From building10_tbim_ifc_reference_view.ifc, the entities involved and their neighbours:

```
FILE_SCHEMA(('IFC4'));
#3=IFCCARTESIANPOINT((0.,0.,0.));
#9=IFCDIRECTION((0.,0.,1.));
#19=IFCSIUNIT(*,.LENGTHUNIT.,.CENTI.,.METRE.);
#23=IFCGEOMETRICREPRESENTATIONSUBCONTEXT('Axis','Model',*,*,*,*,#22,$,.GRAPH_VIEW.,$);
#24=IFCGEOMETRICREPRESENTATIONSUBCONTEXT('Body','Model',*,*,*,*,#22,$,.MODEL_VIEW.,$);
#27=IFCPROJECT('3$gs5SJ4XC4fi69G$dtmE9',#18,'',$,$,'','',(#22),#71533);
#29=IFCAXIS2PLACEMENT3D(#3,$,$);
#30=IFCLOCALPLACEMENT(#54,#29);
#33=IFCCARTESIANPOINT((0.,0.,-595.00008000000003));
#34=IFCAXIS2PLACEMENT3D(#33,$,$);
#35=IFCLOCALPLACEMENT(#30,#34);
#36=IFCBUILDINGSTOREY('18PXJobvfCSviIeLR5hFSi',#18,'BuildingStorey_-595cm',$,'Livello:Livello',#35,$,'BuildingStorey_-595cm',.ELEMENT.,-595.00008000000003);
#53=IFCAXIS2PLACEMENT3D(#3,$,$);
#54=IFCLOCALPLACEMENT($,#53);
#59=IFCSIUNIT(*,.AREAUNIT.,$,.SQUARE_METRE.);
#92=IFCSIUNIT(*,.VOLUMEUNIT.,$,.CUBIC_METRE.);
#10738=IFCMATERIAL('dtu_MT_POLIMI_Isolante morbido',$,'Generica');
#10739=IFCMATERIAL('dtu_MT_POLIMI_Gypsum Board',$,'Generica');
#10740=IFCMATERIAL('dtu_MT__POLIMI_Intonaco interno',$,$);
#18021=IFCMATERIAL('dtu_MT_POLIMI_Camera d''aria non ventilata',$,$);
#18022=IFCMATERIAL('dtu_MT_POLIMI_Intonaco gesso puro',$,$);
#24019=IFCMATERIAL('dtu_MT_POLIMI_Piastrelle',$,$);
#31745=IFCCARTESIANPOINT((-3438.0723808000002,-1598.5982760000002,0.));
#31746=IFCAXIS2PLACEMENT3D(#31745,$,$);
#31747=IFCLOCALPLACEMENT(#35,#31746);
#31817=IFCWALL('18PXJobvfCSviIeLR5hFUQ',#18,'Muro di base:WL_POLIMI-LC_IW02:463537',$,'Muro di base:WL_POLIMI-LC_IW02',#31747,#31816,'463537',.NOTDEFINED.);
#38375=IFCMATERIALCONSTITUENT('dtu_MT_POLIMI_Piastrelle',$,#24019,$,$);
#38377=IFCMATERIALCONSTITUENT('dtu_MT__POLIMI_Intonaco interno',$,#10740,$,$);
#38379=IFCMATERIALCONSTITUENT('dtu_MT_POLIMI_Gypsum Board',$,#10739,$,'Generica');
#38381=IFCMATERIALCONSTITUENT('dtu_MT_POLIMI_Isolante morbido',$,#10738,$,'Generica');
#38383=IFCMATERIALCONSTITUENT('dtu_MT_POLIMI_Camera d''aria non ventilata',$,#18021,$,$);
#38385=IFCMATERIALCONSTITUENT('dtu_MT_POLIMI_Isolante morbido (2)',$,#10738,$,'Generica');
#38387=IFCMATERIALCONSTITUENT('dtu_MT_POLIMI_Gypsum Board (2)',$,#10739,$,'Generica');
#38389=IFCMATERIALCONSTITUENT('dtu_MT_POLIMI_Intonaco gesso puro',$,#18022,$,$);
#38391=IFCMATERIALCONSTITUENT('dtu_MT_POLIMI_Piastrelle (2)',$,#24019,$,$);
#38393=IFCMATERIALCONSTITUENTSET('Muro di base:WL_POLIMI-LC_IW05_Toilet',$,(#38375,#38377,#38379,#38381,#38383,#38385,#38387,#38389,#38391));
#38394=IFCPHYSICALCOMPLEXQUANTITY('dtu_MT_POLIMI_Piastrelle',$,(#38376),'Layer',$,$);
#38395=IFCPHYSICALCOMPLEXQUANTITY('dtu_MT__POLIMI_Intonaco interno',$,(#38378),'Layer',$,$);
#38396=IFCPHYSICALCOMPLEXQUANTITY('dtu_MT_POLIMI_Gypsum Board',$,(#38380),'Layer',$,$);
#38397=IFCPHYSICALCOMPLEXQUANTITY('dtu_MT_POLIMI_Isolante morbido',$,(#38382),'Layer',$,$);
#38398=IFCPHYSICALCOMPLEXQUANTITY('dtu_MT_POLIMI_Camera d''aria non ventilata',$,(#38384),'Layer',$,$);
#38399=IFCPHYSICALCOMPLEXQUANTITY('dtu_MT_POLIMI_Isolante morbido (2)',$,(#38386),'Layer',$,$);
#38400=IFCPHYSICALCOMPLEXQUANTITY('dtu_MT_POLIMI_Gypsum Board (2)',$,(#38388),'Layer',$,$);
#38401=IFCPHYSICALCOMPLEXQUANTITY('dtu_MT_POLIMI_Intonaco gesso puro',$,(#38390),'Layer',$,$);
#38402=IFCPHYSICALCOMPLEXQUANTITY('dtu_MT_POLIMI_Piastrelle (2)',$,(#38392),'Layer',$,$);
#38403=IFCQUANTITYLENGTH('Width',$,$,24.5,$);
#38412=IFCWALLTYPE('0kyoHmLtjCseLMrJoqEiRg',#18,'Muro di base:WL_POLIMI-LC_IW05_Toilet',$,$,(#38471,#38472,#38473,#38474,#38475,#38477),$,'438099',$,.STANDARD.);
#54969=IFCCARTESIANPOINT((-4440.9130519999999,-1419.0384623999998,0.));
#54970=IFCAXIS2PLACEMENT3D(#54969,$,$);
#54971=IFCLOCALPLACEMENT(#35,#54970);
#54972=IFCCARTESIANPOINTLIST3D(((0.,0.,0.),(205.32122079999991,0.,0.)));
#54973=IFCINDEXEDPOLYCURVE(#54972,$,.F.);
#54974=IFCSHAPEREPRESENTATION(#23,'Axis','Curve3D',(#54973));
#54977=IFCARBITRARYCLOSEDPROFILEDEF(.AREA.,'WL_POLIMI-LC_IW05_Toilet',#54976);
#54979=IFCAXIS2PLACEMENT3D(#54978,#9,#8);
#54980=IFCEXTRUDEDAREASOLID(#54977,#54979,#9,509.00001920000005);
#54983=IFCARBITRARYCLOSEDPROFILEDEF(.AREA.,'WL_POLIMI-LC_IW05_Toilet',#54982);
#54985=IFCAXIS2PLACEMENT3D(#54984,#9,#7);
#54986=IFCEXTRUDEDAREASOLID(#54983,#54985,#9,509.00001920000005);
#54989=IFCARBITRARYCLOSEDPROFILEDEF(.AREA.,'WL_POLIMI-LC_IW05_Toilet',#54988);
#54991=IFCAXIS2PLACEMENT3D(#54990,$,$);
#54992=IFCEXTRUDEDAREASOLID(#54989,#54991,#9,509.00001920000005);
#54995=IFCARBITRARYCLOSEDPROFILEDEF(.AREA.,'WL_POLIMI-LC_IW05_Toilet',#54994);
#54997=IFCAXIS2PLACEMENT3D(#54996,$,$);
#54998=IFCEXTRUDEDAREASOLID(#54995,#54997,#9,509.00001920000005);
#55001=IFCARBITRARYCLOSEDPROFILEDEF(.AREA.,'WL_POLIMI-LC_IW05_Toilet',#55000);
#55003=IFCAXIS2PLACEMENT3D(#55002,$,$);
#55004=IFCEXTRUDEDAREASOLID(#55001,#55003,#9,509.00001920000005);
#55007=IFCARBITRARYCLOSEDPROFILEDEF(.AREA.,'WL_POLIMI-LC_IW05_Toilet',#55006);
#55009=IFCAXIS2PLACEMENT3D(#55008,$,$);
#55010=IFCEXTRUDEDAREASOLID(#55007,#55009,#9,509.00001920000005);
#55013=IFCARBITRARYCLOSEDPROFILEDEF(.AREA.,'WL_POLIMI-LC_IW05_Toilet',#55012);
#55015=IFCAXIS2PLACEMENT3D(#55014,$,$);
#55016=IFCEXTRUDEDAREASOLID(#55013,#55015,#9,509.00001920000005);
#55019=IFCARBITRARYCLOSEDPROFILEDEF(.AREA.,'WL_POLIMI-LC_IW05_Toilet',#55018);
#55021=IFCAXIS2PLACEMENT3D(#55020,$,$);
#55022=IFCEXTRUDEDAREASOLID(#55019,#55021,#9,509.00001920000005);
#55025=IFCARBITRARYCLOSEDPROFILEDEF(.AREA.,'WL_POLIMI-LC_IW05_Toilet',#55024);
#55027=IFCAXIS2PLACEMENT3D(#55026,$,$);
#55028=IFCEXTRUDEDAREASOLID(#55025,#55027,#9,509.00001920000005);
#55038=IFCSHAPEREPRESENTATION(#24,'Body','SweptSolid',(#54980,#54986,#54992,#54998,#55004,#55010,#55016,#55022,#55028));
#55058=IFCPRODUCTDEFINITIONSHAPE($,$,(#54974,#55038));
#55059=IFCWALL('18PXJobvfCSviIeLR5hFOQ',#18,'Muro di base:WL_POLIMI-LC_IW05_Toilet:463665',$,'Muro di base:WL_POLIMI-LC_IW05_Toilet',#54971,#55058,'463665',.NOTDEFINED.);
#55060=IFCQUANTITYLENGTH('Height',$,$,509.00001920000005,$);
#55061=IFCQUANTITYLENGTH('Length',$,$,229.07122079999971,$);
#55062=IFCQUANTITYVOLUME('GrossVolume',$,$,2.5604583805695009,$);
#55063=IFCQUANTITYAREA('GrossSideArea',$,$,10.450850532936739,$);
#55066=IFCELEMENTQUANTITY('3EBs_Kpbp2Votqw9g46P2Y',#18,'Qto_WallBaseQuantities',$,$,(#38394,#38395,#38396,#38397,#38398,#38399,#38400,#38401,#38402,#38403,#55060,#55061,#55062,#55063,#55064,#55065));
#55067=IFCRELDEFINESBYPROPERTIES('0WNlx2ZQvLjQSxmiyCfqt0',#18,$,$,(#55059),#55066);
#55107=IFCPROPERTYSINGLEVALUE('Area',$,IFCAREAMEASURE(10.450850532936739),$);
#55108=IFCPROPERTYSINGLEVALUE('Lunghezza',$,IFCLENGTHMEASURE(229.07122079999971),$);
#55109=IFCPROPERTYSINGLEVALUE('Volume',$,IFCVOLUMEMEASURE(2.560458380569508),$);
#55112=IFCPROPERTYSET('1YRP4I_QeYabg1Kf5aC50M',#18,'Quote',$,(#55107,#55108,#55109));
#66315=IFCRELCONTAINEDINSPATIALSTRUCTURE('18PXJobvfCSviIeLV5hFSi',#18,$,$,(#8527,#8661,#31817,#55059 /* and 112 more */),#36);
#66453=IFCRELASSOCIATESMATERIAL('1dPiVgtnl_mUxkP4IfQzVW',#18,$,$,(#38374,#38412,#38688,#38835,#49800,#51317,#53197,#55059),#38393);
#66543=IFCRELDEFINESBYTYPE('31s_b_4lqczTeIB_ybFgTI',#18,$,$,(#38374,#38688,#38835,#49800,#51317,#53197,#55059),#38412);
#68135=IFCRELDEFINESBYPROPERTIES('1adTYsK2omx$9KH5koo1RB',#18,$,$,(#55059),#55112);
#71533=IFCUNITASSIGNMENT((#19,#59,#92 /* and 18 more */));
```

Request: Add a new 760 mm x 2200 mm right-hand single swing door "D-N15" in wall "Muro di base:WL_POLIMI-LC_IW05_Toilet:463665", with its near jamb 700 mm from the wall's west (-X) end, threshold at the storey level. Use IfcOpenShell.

```python
import numpy as np
import ifcopenshell
import ifcopenshell.api.feature
import ifcopenshell.api.geometry
import ifcopenshell.api.pset
import ifcopenshell.api.root
import ifcopenshell.api.spatial
import ifcopenshell.geom
import ifcopenshell.util.element
import ifcopenshell.util.placement
import ifcopenshell.util.representation
import ifcopenshell.util.shape
import ifcopenshell.util.unit

model = ifcopenshell.open("building10_tbim_ifc_reference_view.ifc")
unit_scale = ifcopenshell.util.unit.calculate_unit_scale(model)
area_scale = ifcopenshell.util.unit.calculate_unit_scale(model, "AREAUNIT")
volume_scale = ifcopenshell.util.unit.calculate_unit_scale(model, "VOLUMEUNIT")
settings = ifcopenshell.geom.settings()


def volume(element):
    """Net volume in cubic metres, openings subtracted."""
    shape = ifcopenshell.geom.create_shape(settings, element)
    return ifcopenshell.util.shape.get_volume(shape.geometry)


wall = model.by_guid("18PXJobvfCSviIeLR5hFOQ")
storey = ifcopenshell.util.element.get_container(wall, ifc_class="IfcBuildingStorey")
context = ifcopenshell.util.representation.get_context(model, "Model", "Body", "MODEL_VIEW")
before = volume(wall)

width, height, from_end, sill = 0.76, 2.2, 0.7, 0.0  # metres

# The wall runs along its own X axis, and the end named is its -X end.
wall_shape = ifcopenshell.geom.create_shape(settings, wall)
x, y, z = ifcopenshell.util.shape.get_vertices(wall_shape.geometry).T
start = x.min() + from_end
face, thickness = float(y.min()), float(y.max() - y.min())
wall_matrix = ifcopenshell.util.placement.get_local_placement(wall.ObjectPlacement)
level = ifcopenshell.util.placement.get_local_placement(storey.ObjectPlacement)[2, 3]


def in_wall(x, y):
    """Placement at x, y metres in the wall's axes, at sill height."""
    matrix = wall_matrix.copy()
    matrix[:, 3] = wall_matrix @ np.array([x / unit_scale, y / unit_scale, 0.0, 1.0])
    matrix[2, 3] = level + sill / unit_scale
    return matrix


# Opening: a box that overshoots both wall faces by 50 mm.
opening = ifcopenshell.api.root.create_entity(model, ifc_class="IfcOpeningElement", predefined_type="OPENING")
box = ifcopenshell.api.geometry.add_wall_representation(
    model, context=context, length=width, height=height, thickness=thickness + 0.1
)
ifcopenshell.api.geometry.assign_representation(model, product=opening, representation=box)
ifcopenshell.api.geometry.edit_object_placement(model, product=opening, matrix=in_wall(start, face - 0.05), is_si=False)
ifcopenshell.api.feature.add_feature(model, feature=opening, element=wall)

door = ifcopenshell.api.root.create_entity(model, ifc_class="IfcDoor", name="D-N15", predefined_type="DOOR")
door.OverallWidth, door.OverallHeight = width / unit_scale, height / unit_scale
door.OperationType = "SINGLE_SWING_RIGHT"
body = ifcopenshell.api.geometry.add_door_representation(
    model,
    context=context,
    overall_width=door.OverallWidth,
    overall_height=door.OverallHeight,
    operation_type="SINGLE_SWING_RIGHT",
    lining_properties={"LiningDepth": thickness / unit_scale, "ThresholdDepth": thickness / unit_scale},
)
ifcopenshell.api.geometry.assign_representation(model, product=door, representation=body)
ifcopenshell.api.spatial.assign_container(model, products=[door], relating_structure=storey)
ifcopenshell.api.feature.add_filling(model, opening=opening, element=door)

# The lining spans the wall, so the door starts at the wall face.
ifcopenshell.api.geometry.edit_object_placement(model, product=door, matrix=in_wall(start, face), is_si=False)

after = volume(wall)

# Update the wall's stored quantities.
qto = model.by_id(ifcopenshell.util.element.get_pset(wall, "Qto_WallBaseQuantities", should_inherit=False)["id"])
ifcopenshell.api.pset.edit_qto(model, qto=qto, properties={
    "NetSideArea": after / thickness / area_scale,
    "NetVolume": after / volume_scale,
})
pset = model.by_id(ifcopenshell.util.element.get_pset(wall, "Quote", should_inherit=False)["id"])
ifcopenshell.api.pset.edit_pset(model, pset=pset, properties={
    "Area": model.create_entity("IfcAreaMeasure", after / thickness / area_scale),
    "Volume": model.create_entity("IfcVolumeMeasure", after / volume_scale),
})

print(f"wall volume {before:.3f} -> {after:.3f} m3")

model.write("building10_tbim_ifc_reference_view_edited.ifc")
```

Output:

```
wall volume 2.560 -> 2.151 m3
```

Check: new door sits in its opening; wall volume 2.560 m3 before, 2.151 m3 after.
